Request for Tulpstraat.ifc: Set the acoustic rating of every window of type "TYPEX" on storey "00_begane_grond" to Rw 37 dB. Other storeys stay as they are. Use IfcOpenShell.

First a look at what the model holds.

```python
import ifcopenshell
import ifcopenshell.util.element

model = ifcopenshell.open("Tulpstraat.ifc")
print(model.schema)
storey = next(s for s in model.by_type("IfcBuildingStorey") if s.Name == "00_begane_grond")
windows = [e for e in ifcopenshell.util.element.get_decomposition(storey) if e.is_a("IfcWindow")]
seen = {}
for e in windows:
    element_type = ifcopenshell.util.element.get_type(e)
    key = (element_type.Name if element_type != e and element_type else None, ifcopenshell.util.element.get_pset(e, "Pset_WindowCommon", "AcousticRating"))
    seen[key] = seen.get(key, 0) + 1
for (name, value), count in sorted(seen.items(), key=str):
    print(count, "x", name, "|", value)
```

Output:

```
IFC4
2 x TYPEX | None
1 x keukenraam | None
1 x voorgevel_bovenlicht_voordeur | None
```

```python
import ifcopenshell
import ifcopenshell.api.pset
import ifcopenshell.util.element

model = ifcopenshell.open("Tulpstraat.ifc")

storey = next(s for s in model.by_type("IfcBuildingStorey") if s.Name == "00_begane_grond")
windows = [e for e in ifcopenshell.util.element.get_decomposition(storey) if e.is_a("IfcWindow")]

count = 0
for e in windows:
    element_type = ifcopenshell.util.element.get_type(e)
    if element_type in (None, e) or element_type.Name != "TYPEX":
        continue
    # add_pset returns the element's existing set when there is one.
    pset = ifcopenshell.api.pset.add_pset(model, product=e, name="Pset_WindowCommon")
    ifcopenshell.api.pset.edit_pset(model, pset=pset, properties={"AcousticRating": "Rw 37 dB"})
    count += 1

print(count, "windows updated")

model.write("Tulpstraat_edited.ifc")
```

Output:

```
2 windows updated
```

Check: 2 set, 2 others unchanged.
